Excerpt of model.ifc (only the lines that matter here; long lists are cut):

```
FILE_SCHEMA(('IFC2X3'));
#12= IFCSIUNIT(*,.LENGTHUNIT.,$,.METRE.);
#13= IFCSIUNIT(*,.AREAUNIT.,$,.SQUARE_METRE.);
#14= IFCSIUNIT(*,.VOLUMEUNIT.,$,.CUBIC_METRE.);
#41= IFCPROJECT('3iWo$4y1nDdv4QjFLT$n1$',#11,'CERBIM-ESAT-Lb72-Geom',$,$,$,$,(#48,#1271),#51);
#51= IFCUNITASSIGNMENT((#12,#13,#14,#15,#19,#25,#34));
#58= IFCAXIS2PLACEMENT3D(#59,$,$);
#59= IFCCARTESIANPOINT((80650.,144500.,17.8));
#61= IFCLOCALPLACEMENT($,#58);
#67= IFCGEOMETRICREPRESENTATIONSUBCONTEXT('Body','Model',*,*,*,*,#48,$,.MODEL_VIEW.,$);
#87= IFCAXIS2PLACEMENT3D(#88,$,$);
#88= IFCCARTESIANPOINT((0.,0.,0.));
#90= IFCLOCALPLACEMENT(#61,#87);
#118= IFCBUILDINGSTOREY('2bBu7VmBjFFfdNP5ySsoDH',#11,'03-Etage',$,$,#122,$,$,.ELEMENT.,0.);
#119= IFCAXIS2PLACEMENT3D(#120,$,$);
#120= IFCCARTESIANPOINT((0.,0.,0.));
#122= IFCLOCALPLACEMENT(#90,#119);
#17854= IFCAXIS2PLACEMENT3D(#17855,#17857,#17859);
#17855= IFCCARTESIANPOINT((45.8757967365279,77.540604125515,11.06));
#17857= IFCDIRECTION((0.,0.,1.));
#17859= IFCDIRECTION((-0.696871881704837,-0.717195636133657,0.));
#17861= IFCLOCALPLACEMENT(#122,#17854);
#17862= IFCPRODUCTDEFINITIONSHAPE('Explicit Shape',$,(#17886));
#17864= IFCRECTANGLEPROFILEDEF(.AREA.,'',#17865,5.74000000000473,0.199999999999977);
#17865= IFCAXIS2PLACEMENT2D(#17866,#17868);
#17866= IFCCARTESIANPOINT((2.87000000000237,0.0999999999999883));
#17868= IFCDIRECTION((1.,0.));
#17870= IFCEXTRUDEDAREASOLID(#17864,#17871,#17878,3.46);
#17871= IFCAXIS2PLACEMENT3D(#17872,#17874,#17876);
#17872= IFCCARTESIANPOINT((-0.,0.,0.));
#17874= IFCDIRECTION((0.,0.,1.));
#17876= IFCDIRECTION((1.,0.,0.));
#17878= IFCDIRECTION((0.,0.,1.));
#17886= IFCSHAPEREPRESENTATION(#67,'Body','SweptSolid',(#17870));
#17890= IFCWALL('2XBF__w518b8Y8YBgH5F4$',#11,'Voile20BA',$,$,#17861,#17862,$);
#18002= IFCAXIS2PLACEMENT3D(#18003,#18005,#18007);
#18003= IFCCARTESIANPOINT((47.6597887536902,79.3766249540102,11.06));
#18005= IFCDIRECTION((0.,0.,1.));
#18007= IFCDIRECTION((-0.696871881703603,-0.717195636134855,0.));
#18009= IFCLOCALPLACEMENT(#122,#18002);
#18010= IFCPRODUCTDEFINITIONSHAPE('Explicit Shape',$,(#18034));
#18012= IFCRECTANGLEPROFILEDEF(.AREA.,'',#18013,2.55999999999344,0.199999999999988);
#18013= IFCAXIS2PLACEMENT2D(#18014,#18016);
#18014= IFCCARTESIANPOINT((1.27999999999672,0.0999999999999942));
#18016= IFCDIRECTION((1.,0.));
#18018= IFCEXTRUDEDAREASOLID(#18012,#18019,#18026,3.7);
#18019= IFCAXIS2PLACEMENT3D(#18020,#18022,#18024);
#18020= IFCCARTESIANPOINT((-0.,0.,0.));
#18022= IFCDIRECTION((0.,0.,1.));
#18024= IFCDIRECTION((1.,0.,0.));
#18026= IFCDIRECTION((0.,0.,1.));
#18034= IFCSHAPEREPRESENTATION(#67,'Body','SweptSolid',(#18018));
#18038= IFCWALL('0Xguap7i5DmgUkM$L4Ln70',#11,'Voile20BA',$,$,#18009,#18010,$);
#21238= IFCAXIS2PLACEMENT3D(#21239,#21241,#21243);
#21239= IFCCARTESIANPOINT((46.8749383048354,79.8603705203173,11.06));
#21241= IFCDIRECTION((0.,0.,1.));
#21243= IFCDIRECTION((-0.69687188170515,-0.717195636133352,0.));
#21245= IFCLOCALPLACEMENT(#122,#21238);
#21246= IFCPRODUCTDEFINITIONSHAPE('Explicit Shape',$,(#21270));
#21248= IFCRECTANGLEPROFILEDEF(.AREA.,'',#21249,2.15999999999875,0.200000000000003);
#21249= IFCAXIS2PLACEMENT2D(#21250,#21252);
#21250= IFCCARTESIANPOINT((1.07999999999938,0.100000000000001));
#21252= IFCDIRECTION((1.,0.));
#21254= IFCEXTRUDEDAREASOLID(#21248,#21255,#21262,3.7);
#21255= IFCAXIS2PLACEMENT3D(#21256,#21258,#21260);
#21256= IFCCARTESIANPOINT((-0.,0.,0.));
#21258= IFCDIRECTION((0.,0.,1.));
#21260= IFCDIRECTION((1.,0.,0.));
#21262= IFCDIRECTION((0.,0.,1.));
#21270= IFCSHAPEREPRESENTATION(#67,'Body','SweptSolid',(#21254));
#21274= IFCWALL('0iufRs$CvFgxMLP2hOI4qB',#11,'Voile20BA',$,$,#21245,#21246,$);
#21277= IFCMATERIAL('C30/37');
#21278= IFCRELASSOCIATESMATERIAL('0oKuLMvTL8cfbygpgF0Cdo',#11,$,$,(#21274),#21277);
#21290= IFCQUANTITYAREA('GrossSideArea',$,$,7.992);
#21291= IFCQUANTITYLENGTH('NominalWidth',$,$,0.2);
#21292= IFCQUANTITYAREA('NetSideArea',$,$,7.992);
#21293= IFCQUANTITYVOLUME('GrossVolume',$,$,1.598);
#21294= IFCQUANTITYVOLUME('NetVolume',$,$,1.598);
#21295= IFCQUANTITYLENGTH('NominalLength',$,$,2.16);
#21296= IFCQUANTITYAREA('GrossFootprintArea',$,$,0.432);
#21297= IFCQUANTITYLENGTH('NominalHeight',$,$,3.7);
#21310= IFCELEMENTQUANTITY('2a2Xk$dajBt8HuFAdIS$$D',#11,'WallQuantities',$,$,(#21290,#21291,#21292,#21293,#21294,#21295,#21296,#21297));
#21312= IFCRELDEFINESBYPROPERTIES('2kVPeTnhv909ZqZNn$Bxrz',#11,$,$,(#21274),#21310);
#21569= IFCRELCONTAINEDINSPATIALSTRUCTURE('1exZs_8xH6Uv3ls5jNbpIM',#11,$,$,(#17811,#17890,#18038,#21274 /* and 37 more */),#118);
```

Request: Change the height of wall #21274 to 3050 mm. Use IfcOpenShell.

```python
import ifcopenshell
import ifcopenshell.api.pset
import ifcopenshell.geom
import ifcopenshell.util.element
import ifcopenshell.util.representation
import ifcopenshell.util.shape
import ifcopenshell.util.unit

model = ifcopenshell.open("model.ifc")
unit_scale = ifcopenshell.util.unit.calculate_unit_scale(model)
area_scale = ifcopenshell.util.unit.calculate_unit_scale(model, "AREAUNIT")
volume_scale = ifcopenshell.util.unit.calculate_unit_scale(model, "VOLUMEUNIT")
settings = ifcopenshell.geom.settings()


def volume(element):
    """Net volume in cubic metres, openings subtracted."""
    shape = ifcopenshell.geom.create_shape(settings, element)
    return ifcopenshell.util.shape.get_volume(shape.geometry)


wall = model.by_guid("0iufRs$CvFgxMLP2hOI4qB")
before = volume(wall)

body = ifcopenshell.util.representation.get_representation(wall, "Model", "Body")
solid = body.Items[0]
old_height = solid.Depth
solid.Depth = 3.05 / unit_scale
after = volume(wall)
thickness = 0.2  # wall thickness in metres

# Update the stored height, areas and volumes.
qto = model.by_id(ifcopenshell.util.element.get_pset(wall, "WallQuantities", should_inherit=False)["id"])
ifcopenshell.api.pset.edit_qto(model, qto=qto, properties={
    "GrossSideArea": ifcopenshell.util.element.get_pset(wall, "WallQuantities", "GrossSideArea") * solid.Depth / old_height,
    "NetSideArea": after / thickness / area_scale,
    "GrossVolume": ifcopenshell.util.element.get_pset(wall, "WallQuantities", "GrossVolume") * solid.Depth / old_height,
    "NetVolume": after / volume_scale,
    "NominalHeight": solid.Depth,
})

print(f"height {old_height:g} -> {solid.Depth:g}, volume {before:.3f} -> {after:.3f} m3")

model.write("model_edited.ifc")
```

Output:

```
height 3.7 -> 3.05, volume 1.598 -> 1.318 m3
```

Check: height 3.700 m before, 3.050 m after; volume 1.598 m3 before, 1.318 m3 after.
